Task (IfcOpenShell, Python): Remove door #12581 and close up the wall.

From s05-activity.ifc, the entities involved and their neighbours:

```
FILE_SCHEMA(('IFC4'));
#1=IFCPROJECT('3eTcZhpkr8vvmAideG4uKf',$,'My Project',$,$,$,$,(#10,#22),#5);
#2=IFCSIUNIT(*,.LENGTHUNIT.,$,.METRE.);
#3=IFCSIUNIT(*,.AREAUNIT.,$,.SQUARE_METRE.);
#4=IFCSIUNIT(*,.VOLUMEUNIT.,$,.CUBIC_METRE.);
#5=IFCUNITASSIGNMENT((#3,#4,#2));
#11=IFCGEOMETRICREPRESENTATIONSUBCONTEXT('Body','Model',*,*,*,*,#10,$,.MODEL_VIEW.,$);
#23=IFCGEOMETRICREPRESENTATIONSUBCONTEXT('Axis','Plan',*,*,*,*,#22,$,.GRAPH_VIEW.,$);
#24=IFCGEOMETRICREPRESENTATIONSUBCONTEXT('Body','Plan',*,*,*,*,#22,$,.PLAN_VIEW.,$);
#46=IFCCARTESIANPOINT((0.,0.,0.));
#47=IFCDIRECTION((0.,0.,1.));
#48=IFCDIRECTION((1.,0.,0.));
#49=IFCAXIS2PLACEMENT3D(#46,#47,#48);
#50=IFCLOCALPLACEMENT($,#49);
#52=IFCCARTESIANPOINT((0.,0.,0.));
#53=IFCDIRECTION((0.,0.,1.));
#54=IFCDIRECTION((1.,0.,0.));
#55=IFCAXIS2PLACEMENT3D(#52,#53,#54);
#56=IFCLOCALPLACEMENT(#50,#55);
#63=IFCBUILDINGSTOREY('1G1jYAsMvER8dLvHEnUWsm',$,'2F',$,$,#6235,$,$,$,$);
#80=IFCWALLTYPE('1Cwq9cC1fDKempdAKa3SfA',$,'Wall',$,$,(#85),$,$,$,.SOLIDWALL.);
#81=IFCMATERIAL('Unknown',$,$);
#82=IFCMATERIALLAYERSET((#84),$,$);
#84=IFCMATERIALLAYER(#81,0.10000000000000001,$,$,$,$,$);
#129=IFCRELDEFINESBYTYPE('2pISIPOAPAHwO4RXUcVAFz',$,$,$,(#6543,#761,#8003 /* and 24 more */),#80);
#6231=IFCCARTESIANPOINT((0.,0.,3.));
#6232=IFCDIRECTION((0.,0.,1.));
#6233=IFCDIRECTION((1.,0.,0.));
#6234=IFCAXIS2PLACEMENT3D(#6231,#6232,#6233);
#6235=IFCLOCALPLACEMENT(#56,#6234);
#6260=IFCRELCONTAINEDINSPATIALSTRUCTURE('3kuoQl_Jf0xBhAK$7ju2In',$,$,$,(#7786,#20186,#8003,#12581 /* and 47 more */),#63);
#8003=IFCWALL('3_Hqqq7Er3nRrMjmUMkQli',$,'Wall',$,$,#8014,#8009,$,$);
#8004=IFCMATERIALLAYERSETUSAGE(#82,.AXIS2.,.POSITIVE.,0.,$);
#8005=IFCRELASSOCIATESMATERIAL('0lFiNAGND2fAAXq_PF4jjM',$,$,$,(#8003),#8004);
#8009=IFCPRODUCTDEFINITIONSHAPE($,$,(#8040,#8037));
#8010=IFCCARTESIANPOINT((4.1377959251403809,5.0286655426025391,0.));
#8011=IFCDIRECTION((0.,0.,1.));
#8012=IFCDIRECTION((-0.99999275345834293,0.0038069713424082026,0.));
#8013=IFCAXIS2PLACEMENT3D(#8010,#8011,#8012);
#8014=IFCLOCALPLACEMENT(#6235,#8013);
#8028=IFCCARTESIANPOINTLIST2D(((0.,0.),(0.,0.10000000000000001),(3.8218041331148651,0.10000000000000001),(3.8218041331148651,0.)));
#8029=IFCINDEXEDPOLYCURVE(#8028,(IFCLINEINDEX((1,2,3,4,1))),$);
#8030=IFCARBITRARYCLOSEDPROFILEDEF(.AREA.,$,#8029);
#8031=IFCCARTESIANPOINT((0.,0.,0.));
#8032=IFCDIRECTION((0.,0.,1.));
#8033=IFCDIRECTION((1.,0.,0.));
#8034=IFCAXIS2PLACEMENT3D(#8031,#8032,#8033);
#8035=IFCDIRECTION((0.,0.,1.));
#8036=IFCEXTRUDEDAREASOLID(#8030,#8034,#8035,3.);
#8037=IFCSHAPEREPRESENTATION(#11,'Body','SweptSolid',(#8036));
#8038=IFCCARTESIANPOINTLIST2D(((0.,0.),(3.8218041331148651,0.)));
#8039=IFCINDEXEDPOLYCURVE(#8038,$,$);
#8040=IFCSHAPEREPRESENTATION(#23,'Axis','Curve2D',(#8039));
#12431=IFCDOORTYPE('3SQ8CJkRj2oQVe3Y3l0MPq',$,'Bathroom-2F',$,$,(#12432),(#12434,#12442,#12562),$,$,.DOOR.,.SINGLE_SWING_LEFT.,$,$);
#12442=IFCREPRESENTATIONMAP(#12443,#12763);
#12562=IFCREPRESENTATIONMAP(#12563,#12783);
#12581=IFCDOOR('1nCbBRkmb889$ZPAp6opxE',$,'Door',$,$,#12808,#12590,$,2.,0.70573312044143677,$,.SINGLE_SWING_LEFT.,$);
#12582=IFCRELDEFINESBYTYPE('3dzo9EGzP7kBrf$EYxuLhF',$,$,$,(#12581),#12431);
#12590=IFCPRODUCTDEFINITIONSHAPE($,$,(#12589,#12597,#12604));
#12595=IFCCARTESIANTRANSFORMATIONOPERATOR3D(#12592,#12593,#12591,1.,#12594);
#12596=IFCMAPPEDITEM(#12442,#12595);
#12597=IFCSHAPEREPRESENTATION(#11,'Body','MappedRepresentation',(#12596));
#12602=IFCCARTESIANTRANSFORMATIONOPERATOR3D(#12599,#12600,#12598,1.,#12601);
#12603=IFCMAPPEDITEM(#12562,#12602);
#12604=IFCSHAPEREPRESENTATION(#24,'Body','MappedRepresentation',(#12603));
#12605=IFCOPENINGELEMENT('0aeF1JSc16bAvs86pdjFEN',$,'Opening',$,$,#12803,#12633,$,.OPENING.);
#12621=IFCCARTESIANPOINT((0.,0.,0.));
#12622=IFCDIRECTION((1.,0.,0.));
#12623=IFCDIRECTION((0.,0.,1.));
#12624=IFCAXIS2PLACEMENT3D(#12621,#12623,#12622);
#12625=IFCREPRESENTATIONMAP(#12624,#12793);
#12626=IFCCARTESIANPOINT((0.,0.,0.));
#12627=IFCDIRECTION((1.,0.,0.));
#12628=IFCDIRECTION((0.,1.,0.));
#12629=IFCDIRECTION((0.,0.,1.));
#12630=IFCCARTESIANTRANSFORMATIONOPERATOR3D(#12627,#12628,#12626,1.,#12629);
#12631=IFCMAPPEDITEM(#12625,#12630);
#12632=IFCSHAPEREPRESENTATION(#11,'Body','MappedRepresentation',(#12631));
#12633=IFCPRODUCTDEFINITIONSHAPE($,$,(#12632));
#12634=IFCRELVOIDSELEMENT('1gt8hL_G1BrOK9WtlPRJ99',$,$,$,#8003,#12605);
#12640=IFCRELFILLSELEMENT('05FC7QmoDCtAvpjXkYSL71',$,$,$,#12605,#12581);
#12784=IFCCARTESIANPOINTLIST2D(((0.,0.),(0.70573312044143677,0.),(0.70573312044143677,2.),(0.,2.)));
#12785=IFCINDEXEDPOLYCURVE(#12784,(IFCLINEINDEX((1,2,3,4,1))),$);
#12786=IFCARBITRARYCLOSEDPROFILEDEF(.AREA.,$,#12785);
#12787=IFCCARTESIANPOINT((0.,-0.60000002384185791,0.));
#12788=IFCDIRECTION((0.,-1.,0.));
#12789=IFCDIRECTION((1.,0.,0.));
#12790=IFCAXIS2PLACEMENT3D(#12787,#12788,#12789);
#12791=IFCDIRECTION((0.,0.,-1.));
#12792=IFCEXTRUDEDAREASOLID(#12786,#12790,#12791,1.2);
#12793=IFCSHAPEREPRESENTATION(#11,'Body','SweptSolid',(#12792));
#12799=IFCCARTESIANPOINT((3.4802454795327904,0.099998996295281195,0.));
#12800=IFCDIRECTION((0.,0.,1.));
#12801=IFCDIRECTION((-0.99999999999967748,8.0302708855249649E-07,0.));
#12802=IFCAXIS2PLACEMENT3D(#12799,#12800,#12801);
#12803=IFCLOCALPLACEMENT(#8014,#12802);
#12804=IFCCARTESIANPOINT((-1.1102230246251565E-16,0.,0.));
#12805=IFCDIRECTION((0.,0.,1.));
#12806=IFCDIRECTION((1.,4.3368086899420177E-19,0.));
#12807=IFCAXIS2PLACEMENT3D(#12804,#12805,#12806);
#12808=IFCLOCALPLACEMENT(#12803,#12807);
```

```python
import ifcopenshell
import ifcopenshell.api.feature
import ifcopenshell.api.root
import ifcopenshell.geom
import ifcopenshell.util.shape

model = ifcopenshell.open("s05-activity.ifc")
settings = ifcopenshell.geom.settings()


def volume(element):
    """Net volume in cubic metres, openings subtracted."""
    shape = ifcopenshell.geom.create_shape(settings, element)
    return ifcopenshell.util.shape.get_volume(shape.geometry)


door = model.by_id(12581)
opening = door.FillsVoids[0].RelatingOpeningElement
wall = opening.VoidsElements[0].RelatingBuildingElement
before = volume(wall)

ifcopenshell.api.root.remove_product(model, product=door)
ifcopenshell.api.feature.remove_feature(model, feature=opening)

after = volume(wall)

print(f"wall volume {before:.3f} -> {after:.3f} m3")

model.write("s05-activity_edited.ifc")
```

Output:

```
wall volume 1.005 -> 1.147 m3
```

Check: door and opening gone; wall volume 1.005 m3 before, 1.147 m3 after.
